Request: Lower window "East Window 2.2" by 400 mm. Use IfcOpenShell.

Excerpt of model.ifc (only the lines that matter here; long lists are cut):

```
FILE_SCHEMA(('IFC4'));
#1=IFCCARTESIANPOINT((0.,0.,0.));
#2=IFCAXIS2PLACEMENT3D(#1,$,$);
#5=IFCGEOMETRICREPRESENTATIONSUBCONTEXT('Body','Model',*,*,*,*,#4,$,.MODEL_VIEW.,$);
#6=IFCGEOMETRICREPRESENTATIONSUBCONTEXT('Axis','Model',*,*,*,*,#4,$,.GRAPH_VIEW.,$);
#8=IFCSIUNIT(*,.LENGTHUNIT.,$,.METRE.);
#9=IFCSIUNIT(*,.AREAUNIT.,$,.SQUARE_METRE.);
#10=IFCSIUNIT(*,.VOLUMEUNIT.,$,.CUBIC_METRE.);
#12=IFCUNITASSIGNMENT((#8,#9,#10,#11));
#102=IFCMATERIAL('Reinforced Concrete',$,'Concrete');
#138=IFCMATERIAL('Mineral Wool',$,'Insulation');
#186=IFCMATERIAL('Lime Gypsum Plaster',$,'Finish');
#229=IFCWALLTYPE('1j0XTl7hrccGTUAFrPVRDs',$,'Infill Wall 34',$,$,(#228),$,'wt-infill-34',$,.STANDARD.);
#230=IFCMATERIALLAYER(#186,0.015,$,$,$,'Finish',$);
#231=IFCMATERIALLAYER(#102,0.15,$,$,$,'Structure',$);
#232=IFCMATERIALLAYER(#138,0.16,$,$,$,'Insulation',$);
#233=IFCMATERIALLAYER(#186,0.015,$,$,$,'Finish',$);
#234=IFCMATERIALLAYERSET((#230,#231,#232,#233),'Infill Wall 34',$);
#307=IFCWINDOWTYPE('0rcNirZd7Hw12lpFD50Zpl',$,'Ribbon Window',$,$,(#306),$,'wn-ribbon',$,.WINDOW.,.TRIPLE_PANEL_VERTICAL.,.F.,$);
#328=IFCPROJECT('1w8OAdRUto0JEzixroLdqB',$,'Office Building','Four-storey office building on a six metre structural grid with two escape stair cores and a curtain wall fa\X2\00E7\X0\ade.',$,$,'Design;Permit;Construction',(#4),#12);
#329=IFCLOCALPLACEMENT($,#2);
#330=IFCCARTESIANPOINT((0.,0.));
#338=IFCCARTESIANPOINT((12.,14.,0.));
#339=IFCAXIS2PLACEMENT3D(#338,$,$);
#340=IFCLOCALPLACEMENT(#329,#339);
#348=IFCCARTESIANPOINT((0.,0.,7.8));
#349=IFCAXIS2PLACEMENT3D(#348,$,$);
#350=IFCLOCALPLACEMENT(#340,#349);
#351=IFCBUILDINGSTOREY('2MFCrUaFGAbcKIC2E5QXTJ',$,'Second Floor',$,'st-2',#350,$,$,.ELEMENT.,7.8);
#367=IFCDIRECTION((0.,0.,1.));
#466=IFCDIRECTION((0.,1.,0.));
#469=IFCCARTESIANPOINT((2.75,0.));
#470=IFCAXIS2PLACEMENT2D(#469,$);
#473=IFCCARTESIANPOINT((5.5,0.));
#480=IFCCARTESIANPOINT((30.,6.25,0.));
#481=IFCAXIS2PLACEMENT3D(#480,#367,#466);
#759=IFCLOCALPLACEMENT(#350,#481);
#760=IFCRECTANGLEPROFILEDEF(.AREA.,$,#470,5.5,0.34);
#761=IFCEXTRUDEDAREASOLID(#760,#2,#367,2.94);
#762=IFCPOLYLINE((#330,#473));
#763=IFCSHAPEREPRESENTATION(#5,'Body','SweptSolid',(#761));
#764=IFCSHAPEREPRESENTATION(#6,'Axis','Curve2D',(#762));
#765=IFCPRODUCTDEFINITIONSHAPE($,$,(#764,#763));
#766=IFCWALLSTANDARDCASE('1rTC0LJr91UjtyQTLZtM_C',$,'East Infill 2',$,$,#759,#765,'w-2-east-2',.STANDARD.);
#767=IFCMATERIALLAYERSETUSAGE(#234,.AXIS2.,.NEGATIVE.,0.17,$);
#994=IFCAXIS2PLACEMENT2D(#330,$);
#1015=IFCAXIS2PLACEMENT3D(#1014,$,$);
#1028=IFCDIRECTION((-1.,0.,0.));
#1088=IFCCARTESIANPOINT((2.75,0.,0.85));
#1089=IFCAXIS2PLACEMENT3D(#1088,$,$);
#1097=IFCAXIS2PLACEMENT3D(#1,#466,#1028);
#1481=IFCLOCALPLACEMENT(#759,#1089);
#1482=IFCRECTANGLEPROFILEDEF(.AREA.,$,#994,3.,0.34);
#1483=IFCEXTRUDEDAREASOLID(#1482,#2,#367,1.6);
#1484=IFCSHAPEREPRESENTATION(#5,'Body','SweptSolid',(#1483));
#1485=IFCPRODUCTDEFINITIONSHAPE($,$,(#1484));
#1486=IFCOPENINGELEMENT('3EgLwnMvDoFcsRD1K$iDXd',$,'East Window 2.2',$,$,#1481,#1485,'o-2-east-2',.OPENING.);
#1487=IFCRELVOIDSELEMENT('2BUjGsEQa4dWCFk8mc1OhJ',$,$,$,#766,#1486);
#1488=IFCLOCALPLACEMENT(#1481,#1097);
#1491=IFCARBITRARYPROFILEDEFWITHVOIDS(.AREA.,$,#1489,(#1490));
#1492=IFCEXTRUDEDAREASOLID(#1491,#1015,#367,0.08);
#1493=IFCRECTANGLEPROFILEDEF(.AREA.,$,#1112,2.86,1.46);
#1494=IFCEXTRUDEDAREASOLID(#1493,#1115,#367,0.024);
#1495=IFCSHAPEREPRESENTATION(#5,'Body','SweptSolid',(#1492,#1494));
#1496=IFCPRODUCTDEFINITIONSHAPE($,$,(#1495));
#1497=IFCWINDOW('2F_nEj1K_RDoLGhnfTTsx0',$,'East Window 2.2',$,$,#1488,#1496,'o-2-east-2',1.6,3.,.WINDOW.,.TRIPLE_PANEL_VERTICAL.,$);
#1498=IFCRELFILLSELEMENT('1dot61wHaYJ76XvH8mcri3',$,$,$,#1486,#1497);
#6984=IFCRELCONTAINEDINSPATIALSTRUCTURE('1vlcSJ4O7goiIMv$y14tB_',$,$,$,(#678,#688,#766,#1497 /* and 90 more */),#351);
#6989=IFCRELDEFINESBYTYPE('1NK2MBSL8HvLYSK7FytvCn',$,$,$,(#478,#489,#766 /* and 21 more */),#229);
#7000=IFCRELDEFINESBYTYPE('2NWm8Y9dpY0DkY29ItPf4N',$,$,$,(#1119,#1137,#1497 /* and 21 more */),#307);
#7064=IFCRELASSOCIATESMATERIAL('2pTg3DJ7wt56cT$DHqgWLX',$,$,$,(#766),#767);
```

```python
import numpy as np
import ifcopenshell
import ifcopenshell.api.geometry
import ifcopenshell.util.placement
import ifcopenshell.util.unit

model = ifcopenshell.open("model.ifc")
unit_scale = ifcopenshell.util.unit.calculate_unit_scale(model)

window = model.by_guid("2F_nEj1K_RDoLGhnfTTsx0")
opening = window.FillsVoids[0].RelatingOpeningElement
dz = -0.4

shift = np.array([0.0, 0.0, dz])
# The window is placed relative to its opening, so it follows when the opening moves.
matrix = ifcopenshell.util.placement.get_local_placement(opening.ObjectPlacement)
matrix[:3, 3] += shift
ifcopenshell.api.geometry.edit_object_placement(
    model, product=opening, matrix=matrix, is_si=False, should_transform_children=True
)

print(f"moved by {dz * unit_scale:+.3f} m")

model.write("model_v2.ifc")
```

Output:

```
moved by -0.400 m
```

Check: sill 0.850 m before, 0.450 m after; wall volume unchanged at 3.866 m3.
